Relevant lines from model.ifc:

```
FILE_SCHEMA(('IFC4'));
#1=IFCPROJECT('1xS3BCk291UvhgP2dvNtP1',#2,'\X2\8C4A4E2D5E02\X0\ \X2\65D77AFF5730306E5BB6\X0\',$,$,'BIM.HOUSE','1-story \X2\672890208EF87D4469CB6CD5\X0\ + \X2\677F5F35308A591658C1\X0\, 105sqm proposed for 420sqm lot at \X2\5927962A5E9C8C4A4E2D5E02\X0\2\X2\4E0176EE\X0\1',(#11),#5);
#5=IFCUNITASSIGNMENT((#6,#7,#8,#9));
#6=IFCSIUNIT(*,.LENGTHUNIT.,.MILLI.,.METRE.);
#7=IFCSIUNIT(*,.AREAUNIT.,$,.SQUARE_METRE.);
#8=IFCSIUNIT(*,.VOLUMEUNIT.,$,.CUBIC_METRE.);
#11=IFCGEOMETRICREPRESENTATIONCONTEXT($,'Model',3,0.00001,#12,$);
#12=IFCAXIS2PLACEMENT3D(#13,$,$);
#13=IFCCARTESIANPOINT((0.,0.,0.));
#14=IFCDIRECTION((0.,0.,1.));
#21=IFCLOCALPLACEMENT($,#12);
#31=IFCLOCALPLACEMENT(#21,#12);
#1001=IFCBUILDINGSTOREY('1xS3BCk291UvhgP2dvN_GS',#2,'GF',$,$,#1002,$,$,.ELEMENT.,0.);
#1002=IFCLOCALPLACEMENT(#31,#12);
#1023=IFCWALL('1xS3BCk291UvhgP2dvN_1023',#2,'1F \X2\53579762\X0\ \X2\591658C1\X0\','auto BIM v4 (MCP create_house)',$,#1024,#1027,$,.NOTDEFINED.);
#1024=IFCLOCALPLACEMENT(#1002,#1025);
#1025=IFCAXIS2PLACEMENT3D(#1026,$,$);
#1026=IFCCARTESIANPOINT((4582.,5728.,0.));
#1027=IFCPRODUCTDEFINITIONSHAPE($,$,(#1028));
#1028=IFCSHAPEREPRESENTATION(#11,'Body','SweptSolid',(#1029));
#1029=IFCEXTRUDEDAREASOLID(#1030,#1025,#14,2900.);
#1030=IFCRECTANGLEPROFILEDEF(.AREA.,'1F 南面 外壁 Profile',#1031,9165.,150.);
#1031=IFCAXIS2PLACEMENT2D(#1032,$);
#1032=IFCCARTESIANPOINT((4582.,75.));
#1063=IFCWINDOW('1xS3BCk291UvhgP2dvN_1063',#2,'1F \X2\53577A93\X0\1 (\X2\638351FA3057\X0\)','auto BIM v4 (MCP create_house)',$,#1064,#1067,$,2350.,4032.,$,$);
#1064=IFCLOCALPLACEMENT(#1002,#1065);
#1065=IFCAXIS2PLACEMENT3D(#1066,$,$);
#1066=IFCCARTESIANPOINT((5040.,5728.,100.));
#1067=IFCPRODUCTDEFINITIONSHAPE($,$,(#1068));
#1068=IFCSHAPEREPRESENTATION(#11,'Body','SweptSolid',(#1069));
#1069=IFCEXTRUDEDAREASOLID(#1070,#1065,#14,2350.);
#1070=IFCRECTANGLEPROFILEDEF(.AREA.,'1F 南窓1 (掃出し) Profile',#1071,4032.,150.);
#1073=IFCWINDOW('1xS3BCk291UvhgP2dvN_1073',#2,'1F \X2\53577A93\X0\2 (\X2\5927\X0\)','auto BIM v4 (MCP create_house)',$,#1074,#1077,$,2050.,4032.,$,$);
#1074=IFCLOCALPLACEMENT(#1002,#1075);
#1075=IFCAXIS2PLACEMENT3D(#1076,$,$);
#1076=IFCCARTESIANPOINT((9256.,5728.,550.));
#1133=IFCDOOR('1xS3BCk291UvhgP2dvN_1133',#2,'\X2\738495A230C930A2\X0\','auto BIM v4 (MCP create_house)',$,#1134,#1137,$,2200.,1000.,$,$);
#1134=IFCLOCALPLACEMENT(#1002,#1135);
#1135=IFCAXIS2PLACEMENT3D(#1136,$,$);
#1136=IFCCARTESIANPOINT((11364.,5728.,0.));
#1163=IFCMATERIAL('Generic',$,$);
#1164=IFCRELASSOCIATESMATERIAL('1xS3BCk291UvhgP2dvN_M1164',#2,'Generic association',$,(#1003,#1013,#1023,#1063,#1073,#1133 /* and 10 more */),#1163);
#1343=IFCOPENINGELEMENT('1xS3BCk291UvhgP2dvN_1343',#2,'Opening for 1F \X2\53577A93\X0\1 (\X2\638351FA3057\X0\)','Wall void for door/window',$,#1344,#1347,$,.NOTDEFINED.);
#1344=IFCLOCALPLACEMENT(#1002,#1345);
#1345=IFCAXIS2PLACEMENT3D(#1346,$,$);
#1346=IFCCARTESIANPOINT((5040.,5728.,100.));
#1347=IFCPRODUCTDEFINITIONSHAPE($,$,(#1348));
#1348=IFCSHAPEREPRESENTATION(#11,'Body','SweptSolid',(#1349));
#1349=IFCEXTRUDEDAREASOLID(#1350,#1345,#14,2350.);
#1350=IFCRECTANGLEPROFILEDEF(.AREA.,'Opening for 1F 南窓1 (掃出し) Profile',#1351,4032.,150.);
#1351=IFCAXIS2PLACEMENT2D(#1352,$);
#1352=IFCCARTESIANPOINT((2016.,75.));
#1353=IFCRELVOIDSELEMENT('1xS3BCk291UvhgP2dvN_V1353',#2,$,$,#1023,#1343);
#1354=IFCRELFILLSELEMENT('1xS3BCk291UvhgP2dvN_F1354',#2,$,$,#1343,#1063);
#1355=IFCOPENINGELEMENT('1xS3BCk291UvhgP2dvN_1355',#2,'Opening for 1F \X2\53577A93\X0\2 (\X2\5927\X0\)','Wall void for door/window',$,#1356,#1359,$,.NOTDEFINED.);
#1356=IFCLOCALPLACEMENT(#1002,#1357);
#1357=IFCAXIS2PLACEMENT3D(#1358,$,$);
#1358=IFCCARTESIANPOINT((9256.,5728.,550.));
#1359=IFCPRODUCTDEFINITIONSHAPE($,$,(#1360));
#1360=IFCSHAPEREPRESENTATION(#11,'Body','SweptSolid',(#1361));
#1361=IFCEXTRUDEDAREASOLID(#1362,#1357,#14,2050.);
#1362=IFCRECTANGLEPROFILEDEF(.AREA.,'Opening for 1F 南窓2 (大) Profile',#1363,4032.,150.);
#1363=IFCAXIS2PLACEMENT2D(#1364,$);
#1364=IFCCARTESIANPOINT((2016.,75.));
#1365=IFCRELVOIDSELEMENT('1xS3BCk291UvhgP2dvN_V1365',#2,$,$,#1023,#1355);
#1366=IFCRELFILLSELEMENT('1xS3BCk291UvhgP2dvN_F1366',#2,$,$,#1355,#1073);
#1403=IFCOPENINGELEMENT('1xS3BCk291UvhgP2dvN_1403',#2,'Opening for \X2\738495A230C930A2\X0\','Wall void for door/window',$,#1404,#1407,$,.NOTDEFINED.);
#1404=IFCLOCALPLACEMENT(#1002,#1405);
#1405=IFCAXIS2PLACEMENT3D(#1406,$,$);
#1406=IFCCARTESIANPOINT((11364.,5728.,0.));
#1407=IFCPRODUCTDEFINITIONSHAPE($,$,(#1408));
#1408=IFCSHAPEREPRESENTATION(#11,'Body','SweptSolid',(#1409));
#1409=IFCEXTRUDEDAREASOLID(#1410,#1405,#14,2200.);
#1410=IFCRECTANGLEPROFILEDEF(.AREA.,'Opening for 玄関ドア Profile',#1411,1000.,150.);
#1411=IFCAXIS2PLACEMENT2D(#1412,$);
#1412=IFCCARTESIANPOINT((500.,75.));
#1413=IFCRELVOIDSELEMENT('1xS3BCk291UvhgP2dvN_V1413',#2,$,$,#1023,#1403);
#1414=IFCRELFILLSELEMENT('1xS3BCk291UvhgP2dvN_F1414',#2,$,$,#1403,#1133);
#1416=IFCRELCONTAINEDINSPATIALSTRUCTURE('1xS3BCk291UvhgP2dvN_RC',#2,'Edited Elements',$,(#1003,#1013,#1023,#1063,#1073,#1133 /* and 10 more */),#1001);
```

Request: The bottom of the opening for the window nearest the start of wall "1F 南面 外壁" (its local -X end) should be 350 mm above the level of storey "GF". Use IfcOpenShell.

```python
import numpy as np
import ifcopenshell
import ifcopenshell.api.geometry
import ifcopenshell.geom
import ifcopenshell.util.element
import ifcopenshell.util.placement
import ifcopenshell.util.shape
import ifcopenshell.util.unit

model = ifcopenshell.open("model.ifc")
unit_scale = ifcopenshell.util.unit.calculate_unit_scale(model)

window = model.by_guid("1xS3BCk291UvhgP2dvN_1063")
opening = window.FillsVoids[0].RelatingOpeningElement
storey = ifcopenshell.util.element.get_container(window, ifc_class="IfcBuildingStorey")
level = ifcopenshell.util.placement.get_local_placement(storey.ObjectPlacement)[2, 3]

# The opening's origin need not be at the sill, so measure its lowest point.
shape = ifcopenshell.geom.create_shape(ifcopenshell.geom.settings(), opening)
bottom = ifcopenshell.util.shape.get_shape_bottom_elevation(shape, shape.geometry) / unit_scale
dz = level + 0.35 / unit_scale - bottom

shift = np.array([0.0, 0.0, dz])
# The window is not placed relative to its opening, so move both.
for product in (opening, window):
    matrix = ifcopenshell.util.placement.get_local_placement(product.ObjectPlacement)
    matrix[:3, 3] += shift
    ifcopenshell.api.geometry.edit_object_placement(model, product=product, matrix=matrix, is_si=False)

print(f"moved by {dz * unit_scale:+.3f} m")

model.write("model_updated.ifc")
```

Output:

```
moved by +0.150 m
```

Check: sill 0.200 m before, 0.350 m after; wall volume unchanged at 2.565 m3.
